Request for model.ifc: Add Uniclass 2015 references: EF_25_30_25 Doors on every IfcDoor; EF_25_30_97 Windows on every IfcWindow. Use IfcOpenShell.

First a look at what the model holds.

```python
import ifcopenshell

model = ifcopenshell.open("model.ifc")
print(model.schema)
print("classifications:", [c.Name for c in model.by_type("IfcClassification")])
for ifc_class in ("IfcDoor", "IfcRoof", "IfcStair", "IfcWall", "IfcWindow"):
    print(ifc_class, len(model.by_type(ifc_class)))
```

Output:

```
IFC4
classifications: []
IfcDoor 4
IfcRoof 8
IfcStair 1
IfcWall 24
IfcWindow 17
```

```python
import ifcopenshell
import ifcopenshell.api.classification

model = ifcopenshell.open("model.ifc")

system = ifcopenshell.api.classification.add_classification(model, classification="Uniclass 2015")

codes = {
    "IfcDoor": ("EF_25_30_25", "Doors"),
    "IfcWindow": ("EF_25_30_97", "Windows"),
}
for ifc_class, (code, name) in codes.items():
    products = model.by_type(ifc_class)
    ifcopenshell.api.classification.add_reference(
        model, products=products, classification=system, identification=code, name=name
    )
    print(code, len(products))

model.write("model_v2.ifc")
```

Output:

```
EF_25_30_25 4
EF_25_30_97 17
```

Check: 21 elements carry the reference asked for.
